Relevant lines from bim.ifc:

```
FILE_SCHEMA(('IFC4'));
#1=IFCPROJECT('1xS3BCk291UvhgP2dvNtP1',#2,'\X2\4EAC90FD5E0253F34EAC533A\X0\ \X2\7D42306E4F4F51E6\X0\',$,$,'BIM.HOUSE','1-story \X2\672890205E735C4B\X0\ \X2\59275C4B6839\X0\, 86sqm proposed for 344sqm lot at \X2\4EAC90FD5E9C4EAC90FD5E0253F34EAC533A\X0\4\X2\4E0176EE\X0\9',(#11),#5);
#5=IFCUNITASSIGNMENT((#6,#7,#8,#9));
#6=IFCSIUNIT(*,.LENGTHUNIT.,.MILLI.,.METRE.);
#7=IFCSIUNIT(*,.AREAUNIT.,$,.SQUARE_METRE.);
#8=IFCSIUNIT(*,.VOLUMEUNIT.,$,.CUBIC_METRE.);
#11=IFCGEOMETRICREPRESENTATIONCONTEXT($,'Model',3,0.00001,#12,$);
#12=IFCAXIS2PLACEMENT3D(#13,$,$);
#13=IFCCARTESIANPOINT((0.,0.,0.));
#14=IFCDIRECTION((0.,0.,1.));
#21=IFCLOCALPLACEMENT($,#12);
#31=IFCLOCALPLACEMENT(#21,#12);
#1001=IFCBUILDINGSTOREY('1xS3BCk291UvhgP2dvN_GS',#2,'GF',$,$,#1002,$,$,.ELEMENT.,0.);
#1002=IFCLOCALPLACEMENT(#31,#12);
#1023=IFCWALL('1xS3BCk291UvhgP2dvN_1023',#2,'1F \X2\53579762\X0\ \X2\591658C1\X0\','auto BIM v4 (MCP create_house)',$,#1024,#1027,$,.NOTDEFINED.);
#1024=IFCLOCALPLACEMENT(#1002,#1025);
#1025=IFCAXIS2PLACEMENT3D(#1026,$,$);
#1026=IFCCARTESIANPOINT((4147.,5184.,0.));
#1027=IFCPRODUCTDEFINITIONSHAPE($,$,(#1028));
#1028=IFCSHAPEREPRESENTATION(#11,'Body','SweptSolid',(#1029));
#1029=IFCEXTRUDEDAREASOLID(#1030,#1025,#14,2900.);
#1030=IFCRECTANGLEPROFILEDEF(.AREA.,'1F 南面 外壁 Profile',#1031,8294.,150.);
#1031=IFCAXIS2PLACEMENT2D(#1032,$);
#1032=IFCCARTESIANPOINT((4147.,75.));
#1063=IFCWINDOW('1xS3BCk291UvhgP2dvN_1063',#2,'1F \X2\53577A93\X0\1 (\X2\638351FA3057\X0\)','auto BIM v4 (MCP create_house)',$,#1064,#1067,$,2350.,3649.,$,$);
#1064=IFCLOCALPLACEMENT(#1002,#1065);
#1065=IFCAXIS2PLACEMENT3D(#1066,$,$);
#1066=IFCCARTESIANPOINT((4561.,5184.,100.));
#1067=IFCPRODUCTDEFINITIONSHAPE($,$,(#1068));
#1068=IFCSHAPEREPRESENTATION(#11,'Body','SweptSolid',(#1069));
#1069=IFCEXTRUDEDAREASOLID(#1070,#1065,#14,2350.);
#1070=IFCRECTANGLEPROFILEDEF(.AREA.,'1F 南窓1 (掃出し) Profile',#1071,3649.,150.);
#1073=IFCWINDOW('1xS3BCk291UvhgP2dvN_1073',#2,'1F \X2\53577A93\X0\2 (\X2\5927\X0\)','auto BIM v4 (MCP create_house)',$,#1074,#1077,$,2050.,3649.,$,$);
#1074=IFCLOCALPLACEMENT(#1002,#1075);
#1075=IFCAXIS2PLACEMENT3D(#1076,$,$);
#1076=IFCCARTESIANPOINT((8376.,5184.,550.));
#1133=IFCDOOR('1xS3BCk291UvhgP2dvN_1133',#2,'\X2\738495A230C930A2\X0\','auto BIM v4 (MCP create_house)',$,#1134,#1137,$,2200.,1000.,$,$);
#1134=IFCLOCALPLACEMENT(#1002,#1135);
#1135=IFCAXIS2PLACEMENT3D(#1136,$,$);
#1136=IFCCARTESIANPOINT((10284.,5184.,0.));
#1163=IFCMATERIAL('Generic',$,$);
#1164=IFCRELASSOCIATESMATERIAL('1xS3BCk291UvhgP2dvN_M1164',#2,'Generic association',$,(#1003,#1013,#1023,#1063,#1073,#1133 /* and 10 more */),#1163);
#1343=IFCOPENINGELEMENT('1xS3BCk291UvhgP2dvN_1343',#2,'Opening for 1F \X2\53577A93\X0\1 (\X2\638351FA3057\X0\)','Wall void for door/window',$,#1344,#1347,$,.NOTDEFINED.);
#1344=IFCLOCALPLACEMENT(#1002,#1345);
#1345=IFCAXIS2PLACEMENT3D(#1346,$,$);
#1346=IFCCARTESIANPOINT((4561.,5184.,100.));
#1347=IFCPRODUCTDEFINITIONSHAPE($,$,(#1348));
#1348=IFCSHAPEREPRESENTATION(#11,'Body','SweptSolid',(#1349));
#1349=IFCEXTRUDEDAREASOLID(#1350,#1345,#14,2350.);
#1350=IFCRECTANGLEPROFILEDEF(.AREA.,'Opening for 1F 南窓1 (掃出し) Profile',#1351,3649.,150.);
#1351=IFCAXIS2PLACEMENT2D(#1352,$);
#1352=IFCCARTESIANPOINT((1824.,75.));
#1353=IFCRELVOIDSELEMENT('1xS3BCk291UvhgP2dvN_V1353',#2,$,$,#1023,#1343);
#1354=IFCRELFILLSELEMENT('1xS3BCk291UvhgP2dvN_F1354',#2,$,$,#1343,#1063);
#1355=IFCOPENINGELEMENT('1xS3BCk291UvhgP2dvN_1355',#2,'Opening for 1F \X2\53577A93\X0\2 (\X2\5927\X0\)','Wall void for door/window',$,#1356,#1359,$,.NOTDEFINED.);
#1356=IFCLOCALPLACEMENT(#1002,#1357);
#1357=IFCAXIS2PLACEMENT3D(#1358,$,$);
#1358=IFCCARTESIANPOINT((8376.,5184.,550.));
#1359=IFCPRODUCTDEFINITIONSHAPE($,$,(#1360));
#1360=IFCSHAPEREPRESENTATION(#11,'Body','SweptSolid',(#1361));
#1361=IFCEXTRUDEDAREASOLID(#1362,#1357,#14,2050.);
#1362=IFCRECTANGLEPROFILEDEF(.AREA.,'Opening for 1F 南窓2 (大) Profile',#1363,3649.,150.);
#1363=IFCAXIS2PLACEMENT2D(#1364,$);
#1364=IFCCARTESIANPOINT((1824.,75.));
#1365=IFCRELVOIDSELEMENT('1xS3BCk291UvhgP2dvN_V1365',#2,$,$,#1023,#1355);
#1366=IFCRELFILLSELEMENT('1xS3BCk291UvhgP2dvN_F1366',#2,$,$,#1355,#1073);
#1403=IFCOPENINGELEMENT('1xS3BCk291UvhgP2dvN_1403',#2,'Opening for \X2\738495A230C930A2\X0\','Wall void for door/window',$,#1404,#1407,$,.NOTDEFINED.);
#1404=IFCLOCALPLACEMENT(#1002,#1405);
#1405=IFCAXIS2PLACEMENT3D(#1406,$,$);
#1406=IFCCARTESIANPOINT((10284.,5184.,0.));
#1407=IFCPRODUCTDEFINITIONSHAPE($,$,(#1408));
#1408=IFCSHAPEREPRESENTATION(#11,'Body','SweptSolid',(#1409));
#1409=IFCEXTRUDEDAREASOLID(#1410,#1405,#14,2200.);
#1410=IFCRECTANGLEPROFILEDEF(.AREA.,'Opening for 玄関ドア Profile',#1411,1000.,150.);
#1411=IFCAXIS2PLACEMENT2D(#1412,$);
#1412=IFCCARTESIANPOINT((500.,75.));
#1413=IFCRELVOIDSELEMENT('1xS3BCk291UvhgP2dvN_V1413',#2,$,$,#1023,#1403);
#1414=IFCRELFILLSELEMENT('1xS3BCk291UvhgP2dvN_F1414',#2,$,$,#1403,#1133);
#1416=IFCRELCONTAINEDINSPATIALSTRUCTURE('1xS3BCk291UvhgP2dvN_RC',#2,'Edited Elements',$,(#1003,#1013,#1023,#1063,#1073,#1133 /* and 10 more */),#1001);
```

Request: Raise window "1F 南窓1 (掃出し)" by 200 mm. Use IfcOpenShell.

```python
import numpy as np
import ifcopenshell
import ifcopenshell.api.geometry
import ifcopenshell.util.placement
import ifcopenshell.util.unit

model = ifcopenshell.open("bim.ifc")
unit_scale = ifcopenshell.util.unit.calculate_unit_scale(model)

window = model.by_guid("1xS3BCk291UvhgP2dvN_1063")
opening = window.FillsVoids[0].RelatingOpeningElement
dz = 0.2 / unit_scale

shift = np.array([0.0, 0.0, dz])
# The window is not placed relative to its opening, so move both.
for product in (opening, window):
    matrix = ifcopenshell.util.placement.get_local_placement(product.ObjectPlacement)
    matrix[:3, 3] += shift
    ifcopenshell.api.geometry.edit_object_placement(model, product=product, matrix=matrix, is_si=False)

print(f"moved by {dz * unit_scale:+.3f} m")

model.write("bim_rev.ifc")
```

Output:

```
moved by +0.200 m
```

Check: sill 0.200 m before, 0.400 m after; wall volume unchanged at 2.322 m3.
